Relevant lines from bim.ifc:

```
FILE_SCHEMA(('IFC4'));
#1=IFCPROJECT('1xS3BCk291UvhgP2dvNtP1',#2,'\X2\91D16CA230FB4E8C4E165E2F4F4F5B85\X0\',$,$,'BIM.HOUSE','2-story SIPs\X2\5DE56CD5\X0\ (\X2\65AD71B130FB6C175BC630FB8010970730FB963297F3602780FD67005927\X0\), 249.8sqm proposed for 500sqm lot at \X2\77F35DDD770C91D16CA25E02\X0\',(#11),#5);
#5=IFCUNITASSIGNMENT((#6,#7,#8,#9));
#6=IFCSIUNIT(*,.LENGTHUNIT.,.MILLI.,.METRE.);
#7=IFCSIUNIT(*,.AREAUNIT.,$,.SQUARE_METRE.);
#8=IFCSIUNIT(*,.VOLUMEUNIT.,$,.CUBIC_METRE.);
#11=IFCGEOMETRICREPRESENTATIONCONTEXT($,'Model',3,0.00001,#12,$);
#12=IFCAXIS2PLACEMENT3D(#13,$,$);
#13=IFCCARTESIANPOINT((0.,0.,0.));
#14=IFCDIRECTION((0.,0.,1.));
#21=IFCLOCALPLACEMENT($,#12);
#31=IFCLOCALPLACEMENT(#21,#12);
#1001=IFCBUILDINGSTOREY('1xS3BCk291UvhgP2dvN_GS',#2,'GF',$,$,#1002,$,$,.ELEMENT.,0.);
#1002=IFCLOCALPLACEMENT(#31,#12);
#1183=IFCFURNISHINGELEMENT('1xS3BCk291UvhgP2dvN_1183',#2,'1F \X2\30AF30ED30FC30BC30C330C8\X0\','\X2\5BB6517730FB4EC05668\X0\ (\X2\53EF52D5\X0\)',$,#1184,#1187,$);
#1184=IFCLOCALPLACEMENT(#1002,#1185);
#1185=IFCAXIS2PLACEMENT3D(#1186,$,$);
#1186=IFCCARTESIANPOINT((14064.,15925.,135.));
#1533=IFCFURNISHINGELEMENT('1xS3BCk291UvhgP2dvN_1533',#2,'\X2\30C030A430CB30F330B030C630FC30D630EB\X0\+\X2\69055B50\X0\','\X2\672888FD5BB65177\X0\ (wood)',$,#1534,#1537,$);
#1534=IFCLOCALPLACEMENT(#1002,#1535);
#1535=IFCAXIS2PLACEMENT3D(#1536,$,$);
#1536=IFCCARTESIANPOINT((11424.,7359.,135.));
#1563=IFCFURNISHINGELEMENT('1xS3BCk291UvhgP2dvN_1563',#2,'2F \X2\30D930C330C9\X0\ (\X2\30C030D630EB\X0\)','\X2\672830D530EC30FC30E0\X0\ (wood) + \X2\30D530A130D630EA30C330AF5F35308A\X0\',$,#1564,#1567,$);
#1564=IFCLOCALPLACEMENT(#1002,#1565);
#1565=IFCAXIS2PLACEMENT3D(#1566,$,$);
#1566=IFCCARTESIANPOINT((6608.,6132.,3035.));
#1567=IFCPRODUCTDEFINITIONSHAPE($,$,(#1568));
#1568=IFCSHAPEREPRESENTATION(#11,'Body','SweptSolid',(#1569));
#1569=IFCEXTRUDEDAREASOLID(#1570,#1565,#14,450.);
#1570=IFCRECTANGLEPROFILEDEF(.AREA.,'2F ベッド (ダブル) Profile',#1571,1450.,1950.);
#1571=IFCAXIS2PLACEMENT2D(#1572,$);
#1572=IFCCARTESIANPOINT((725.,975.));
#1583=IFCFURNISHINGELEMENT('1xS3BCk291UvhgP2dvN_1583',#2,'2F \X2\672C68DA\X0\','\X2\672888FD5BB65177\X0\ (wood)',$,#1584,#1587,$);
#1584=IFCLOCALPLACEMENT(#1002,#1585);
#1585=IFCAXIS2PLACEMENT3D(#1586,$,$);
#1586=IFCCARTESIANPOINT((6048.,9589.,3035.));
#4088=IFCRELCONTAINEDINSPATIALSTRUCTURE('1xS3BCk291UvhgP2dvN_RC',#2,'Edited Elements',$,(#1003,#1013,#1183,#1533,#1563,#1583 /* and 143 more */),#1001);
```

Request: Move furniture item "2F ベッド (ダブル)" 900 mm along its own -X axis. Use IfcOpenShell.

```python
import ifcopenshell
import ifcopenshell.api.geometry
import ifcopenshell.util.placement

model = ifcopenshell.open("bim.ifc")

item = model.by_guid("1xS3BCk291UvhgP2dvN_1563")
matrix = ifcopenshell.util.placement.get_local_placement(item.ObjectPlacement)
matrix[:3, 3] -= matrix[:3, 0] * 900.0
ifcopenshell.api.geometry.edit_object_placement(model, product=item, matrix=matrix, is_si=False)

print(ifcopenshell.util.placement.get_local_placement(item.ObjectPlacement).round(3) + 0.0)

model.write("bim-out.ifc")
```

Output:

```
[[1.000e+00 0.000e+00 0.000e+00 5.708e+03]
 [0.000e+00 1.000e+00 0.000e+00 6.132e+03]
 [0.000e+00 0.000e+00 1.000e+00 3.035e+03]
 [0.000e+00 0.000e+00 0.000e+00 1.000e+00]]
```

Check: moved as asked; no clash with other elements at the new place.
